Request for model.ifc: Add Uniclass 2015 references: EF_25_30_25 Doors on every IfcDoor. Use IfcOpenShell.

First a look at what the model holds.

```python
import ifcopenshell

model = ifcopenshell.open("model.ifc")
print(model.schema)
print("classifications:", [c.Name for c in model.by_type("IfcClassification")])
for ifc_class in ("IfcDoor", "IfcRoof", "IfcStair", "IfcWall", "IfcWindow"):
    print(ifc_class, len(model.by_type(ifc_class)))
```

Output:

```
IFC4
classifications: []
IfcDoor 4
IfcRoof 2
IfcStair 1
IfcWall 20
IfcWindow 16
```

```python
import ifcopenshell
import ifcopenshell.api.classification

model = ifcopenshell.open("model.ifc")

system = ifcopenshell.api.classification.add_classification(model, classification="Uniclass 2015")

codes = {
    "IfcDoor": ("EF_25_30_25", "Doors"),
}
for ifc_class, (code, name) in codes.items():
    products = model.by_type(ifc_class)
    ifcopenshell.api.classification.add_reference(
        model, products=products, classification=system, identification=code, name=name
    )
    print(code, len(products))

model.write("model_v2.ifc")
```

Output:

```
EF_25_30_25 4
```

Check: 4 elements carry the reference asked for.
